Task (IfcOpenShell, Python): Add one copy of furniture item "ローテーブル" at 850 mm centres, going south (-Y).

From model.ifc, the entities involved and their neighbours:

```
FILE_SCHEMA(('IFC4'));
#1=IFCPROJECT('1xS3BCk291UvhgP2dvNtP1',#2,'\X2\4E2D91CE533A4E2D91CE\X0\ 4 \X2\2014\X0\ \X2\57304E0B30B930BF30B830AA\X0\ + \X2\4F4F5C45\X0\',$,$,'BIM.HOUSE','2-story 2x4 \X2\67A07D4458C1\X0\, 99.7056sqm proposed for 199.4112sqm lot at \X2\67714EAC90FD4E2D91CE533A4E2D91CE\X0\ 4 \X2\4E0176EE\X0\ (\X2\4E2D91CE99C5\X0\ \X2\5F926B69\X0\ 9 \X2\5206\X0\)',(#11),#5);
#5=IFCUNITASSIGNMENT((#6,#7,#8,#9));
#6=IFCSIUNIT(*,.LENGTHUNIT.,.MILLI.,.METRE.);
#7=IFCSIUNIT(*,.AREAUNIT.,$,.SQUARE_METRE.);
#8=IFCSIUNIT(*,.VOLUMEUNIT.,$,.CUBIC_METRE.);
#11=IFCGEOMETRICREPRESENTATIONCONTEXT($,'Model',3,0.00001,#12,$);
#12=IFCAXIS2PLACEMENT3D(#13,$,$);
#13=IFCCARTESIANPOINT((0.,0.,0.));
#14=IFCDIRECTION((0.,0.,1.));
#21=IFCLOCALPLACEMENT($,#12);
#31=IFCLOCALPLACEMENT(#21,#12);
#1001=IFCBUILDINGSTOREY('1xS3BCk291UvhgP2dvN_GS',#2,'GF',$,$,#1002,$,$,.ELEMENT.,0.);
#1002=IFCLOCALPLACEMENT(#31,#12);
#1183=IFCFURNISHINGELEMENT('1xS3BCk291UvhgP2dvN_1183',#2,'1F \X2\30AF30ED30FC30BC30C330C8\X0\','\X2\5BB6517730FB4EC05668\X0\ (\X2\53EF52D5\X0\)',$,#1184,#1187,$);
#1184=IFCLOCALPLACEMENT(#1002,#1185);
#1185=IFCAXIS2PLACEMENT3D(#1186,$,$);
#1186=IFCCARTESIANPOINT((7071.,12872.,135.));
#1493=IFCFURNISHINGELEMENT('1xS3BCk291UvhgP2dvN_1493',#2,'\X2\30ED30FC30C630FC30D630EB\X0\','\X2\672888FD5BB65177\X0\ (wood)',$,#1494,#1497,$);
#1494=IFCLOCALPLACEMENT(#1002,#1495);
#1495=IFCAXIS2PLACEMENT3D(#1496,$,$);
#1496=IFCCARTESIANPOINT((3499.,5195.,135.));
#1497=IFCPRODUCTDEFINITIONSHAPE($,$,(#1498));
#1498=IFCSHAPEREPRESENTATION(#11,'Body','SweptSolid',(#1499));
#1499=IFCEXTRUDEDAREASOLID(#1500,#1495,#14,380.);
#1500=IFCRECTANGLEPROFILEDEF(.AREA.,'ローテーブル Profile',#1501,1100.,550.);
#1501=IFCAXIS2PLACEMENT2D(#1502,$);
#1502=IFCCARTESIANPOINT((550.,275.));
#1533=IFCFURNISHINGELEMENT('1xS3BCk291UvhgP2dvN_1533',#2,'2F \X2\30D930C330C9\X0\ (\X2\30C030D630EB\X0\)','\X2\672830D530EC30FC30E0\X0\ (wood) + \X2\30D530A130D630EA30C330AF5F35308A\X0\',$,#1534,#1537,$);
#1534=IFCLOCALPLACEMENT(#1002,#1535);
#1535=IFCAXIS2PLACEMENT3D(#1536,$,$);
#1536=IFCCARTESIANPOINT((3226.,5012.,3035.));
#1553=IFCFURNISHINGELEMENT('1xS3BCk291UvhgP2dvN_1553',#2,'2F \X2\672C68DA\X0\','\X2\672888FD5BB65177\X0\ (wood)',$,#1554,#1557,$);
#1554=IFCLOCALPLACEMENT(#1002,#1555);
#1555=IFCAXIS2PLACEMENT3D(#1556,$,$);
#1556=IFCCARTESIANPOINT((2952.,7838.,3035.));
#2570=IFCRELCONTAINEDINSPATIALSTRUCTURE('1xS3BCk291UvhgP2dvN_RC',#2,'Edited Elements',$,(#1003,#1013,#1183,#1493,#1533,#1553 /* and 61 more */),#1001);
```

```python
import numpy as np
import ifcopenshell
import ifcopenshell.api.geometry
import ifcopenshell.api.root
import ifcopenshell.util.element
import ifcopenshell.util.placement

model = ifcopenshell.open("model.ifc")


def reuse_history(source, copy):
    """copy_class also copies each property set's owner history, people and application; keep the originals."""
    for rel in copy.IsDefinedBy:
        if rel.is_a("IfcRelDefinesByProperties") and (history := rel.RelatingPropertyDefinition.OwnerHistory):
            rel.RelatingPropertyDefinition.OwnerHistory = source.OwnerHistory
            ifcopenshell.util.element.remove_deep2(model, history)


source = model.by_guid("1xS3BCk291UvhgP2dvN_1493")
base = ifcopenshell.util.placement.get_local_placement(source.ObjectPlacement)
step = np.array([0.0, -1.0, 0.0]) * 850.0

for i in range(1, 2):
    copy = ifcopenshell.api.root.copy_class(model, product=source)
    copy.Representation = ifcopenshell.util.element.copy_deep(
        model, source.Representation, exclude=["IfcGeometricRepresentationContext", "IfcRepresentationMap"]
    )
    reuse_history(source, copy)
    matrix = base.copy()
    matrix[:3, 3] += i * step
    print("added at", matrix[:3, 3].round(3) + 0.0)
    ifcopenshell.api.geometry.edit_object_placement(model, product=copy, matrix=matrix, is_si=False)

model.write("model_rev.ifc")
```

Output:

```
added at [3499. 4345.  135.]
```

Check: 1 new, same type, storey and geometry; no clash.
